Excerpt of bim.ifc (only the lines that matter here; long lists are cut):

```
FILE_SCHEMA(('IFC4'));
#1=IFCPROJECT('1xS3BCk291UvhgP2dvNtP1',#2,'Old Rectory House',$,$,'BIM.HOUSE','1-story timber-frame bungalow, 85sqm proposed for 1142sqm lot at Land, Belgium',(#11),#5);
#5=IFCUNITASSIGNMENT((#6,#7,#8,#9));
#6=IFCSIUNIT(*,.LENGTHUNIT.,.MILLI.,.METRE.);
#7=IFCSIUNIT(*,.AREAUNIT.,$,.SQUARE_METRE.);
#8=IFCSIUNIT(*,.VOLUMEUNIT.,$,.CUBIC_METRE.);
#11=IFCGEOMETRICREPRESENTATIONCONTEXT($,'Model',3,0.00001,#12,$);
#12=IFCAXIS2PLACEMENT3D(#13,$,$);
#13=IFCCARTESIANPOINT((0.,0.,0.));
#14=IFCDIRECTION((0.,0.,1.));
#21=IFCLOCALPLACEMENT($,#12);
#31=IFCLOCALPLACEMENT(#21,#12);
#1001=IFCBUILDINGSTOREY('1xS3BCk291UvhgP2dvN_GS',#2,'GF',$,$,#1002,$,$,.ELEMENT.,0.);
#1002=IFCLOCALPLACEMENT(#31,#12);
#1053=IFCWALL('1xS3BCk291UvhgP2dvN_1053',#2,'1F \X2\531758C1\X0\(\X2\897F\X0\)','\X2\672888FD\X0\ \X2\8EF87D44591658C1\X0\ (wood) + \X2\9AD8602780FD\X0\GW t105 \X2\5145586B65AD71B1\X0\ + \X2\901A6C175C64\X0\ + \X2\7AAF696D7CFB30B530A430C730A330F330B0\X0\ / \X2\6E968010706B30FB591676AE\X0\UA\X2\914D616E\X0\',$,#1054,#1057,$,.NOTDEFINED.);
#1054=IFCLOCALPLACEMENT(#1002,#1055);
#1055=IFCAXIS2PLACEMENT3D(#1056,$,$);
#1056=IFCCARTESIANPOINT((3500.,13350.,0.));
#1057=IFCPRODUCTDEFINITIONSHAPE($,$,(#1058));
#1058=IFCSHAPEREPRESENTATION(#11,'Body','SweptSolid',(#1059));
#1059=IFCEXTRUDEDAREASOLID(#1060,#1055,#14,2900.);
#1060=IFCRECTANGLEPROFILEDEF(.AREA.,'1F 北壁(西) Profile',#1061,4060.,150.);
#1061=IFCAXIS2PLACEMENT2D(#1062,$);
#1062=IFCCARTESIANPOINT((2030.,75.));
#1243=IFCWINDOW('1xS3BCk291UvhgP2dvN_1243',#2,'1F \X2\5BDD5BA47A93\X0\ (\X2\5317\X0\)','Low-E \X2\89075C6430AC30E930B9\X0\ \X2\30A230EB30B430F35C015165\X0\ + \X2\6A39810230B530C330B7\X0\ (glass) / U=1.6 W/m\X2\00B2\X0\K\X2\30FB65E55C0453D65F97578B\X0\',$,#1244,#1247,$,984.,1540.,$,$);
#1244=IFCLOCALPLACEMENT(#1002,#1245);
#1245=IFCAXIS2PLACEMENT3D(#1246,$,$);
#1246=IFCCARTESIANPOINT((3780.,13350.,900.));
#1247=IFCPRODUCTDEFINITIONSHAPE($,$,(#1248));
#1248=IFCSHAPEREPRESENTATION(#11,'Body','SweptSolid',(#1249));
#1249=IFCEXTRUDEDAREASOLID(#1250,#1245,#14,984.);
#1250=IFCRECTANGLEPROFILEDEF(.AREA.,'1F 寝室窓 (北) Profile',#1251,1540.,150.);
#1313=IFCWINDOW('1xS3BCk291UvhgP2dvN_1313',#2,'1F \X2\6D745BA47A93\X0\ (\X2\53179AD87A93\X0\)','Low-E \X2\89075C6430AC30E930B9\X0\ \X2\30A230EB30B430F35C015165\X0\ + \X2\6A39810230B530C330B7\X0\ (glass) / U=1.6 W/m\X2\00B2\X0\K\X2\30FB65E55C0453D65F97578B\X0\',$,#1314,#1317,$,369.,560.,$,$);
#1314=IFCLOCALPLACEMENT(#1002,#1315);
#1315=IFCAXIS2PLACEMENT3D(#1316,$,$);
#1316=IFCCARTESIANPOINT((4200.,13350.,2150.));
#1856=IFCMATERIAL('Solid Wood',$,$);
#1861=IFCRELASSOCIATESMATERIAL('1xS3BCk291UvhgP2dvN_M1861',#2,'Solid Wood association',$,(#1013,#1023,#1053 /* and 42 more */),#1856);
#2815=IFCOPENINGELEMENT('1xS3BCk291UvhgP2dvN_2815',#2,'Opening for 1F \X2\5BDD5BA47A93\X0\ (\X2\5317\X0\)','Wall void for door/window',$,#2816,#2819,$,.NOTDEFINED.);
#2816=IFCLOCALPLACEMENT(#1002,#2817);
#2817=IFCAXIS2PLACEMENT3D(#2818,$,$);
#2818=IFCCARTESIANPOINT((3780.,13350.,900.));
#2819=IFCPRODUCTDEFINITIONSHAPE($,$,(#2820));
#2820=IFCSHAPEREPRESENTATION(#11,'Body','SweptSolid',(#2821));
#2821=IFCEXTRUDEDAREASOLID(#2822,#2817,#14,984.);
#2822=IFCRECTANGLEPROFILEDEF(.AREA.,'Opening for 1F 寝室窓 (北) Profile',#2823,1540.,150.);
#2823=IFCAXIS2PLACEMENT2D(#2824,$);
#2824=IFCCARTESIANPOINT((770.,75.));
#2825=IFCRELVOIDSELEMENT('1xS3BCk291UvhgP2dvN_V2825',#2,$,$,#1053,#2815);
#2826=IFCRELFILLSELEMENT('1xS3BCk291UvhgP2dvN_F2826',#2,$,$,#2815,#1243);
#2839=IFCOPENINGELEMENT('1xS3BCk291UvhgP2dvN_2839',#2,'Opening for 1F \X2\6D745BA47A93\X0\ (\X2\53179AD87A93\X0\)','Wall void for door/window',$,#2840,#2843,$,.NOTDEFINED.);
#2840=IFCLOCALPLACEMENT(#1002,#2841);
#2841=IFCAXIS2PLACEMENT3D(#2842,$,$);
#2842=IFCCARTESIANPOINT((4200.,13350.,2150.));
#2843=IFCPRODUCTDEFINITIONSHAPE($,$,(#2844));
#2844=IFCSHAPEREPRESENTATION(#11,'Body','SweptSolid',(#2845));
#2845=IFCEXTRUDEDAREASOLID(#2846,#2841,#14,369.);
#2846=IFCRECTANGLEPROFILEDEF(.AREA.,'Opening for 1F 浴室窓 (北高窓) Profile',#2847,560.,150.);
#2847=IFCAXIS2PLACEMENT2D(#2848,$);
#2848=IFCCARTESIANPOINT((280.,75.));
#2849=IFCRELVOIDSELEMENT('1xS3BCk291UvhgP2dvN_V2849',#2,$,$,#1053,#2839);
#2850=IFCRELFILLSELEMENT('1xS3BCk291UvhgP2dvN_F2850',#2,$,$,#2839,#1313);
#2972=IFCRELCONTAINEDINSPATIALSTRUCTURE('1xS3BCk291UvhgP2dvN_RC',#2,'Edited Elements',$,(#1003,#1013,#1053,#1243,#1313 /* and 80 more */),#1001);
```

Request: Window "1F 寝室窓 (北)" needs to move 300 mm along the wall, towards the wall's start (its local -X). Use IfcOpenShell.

```python
import ifcopenshell
import ifcopenshell.api.geometry
import ifcopenshell.util.placement

model = ifcopenshell.open("bim.ifc")

window = model.by_guid("1xS3BCk291UvhgP2dvN_1243")
opening = window.FillsVoids[0].RelatingOpeningElement
wall = opening.VoidsElements[0].RelatingBuildingElement

wall_matrix = ifcopenshell.util.placement.get_local_placement(wall.ObjectPlacement)
shift = wall_matrix[:3, 0] * -300.0
before = ifcopenshell.util.placement.get_local_placement(window.ObjectPlacement)[:3, 3].copy()

# The window is not placed relative to its opening, so move both.
for product in (opening, window):
    matrix = ifcopenshell.util.placement.get_local_placement(product.ObjectPlacement)
    matrix[:3, 3] += shift
    ifcopenshell.api.geometry.edit_object_placement(model, product=product, matrix=matrix, is_si=False)

after = ifcopenshell.util.placement.get_local_placement(window.ObjectPlacement)[:3, 3]
print("window moved by", (after - before).round(3) + 0.0)

model.write("bim-out.ifc")
```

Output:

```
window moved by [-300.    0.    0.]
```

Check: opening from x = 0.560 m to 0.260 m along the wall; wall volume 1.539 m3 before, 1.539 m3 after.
